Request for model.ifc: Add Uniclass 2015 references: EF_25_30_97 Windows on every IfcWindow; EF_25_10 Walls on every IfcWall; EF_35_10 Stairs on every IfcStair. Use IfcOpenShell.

First a look at what the model holds.

```python
import ifcopenshell

model = ifcopenshell.open("model.ifc")
print(model.schema)
print("classifications:", [c.Name for c in model.by_type("IfcClassification")])
for ifc_class in ("IfcDoor", "IfcRoof", "IfcStair", "IfcWall", "IfcWindow"):
    print(ifc_class, len(model.by_type(ifc_class)))
```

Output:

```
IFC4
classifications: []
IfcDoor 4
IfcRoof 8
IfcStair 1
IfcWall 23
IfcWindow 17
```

```python
import ifcopenshell
import ifcopenshell.api.classification

model = ifcopenshell.open("model.ifc")

system = ifcopenshell.api.classification.add_classification(model, classification="Uniclass 2015")

codes = {
    "IfcWindow": ("EF_25_30_97", "Windows"),
    "IfcWall": ("EF_25_10", "Walls"),
    "IfcStair": ("EF_35_10", "Stairs"),
}
for ifc_class, (code, name) in codes.items():
    products = model.by_type(ifc_class)
    ifcopenshell.api.classification.add_reference(
        model, products=products, classification=system, identification=code, name=name
    )
    print(code, len(products))

model.write("model_updated.ifc")
```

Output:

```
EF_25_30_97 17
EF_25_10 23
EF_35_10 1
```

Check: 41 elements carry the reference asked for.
